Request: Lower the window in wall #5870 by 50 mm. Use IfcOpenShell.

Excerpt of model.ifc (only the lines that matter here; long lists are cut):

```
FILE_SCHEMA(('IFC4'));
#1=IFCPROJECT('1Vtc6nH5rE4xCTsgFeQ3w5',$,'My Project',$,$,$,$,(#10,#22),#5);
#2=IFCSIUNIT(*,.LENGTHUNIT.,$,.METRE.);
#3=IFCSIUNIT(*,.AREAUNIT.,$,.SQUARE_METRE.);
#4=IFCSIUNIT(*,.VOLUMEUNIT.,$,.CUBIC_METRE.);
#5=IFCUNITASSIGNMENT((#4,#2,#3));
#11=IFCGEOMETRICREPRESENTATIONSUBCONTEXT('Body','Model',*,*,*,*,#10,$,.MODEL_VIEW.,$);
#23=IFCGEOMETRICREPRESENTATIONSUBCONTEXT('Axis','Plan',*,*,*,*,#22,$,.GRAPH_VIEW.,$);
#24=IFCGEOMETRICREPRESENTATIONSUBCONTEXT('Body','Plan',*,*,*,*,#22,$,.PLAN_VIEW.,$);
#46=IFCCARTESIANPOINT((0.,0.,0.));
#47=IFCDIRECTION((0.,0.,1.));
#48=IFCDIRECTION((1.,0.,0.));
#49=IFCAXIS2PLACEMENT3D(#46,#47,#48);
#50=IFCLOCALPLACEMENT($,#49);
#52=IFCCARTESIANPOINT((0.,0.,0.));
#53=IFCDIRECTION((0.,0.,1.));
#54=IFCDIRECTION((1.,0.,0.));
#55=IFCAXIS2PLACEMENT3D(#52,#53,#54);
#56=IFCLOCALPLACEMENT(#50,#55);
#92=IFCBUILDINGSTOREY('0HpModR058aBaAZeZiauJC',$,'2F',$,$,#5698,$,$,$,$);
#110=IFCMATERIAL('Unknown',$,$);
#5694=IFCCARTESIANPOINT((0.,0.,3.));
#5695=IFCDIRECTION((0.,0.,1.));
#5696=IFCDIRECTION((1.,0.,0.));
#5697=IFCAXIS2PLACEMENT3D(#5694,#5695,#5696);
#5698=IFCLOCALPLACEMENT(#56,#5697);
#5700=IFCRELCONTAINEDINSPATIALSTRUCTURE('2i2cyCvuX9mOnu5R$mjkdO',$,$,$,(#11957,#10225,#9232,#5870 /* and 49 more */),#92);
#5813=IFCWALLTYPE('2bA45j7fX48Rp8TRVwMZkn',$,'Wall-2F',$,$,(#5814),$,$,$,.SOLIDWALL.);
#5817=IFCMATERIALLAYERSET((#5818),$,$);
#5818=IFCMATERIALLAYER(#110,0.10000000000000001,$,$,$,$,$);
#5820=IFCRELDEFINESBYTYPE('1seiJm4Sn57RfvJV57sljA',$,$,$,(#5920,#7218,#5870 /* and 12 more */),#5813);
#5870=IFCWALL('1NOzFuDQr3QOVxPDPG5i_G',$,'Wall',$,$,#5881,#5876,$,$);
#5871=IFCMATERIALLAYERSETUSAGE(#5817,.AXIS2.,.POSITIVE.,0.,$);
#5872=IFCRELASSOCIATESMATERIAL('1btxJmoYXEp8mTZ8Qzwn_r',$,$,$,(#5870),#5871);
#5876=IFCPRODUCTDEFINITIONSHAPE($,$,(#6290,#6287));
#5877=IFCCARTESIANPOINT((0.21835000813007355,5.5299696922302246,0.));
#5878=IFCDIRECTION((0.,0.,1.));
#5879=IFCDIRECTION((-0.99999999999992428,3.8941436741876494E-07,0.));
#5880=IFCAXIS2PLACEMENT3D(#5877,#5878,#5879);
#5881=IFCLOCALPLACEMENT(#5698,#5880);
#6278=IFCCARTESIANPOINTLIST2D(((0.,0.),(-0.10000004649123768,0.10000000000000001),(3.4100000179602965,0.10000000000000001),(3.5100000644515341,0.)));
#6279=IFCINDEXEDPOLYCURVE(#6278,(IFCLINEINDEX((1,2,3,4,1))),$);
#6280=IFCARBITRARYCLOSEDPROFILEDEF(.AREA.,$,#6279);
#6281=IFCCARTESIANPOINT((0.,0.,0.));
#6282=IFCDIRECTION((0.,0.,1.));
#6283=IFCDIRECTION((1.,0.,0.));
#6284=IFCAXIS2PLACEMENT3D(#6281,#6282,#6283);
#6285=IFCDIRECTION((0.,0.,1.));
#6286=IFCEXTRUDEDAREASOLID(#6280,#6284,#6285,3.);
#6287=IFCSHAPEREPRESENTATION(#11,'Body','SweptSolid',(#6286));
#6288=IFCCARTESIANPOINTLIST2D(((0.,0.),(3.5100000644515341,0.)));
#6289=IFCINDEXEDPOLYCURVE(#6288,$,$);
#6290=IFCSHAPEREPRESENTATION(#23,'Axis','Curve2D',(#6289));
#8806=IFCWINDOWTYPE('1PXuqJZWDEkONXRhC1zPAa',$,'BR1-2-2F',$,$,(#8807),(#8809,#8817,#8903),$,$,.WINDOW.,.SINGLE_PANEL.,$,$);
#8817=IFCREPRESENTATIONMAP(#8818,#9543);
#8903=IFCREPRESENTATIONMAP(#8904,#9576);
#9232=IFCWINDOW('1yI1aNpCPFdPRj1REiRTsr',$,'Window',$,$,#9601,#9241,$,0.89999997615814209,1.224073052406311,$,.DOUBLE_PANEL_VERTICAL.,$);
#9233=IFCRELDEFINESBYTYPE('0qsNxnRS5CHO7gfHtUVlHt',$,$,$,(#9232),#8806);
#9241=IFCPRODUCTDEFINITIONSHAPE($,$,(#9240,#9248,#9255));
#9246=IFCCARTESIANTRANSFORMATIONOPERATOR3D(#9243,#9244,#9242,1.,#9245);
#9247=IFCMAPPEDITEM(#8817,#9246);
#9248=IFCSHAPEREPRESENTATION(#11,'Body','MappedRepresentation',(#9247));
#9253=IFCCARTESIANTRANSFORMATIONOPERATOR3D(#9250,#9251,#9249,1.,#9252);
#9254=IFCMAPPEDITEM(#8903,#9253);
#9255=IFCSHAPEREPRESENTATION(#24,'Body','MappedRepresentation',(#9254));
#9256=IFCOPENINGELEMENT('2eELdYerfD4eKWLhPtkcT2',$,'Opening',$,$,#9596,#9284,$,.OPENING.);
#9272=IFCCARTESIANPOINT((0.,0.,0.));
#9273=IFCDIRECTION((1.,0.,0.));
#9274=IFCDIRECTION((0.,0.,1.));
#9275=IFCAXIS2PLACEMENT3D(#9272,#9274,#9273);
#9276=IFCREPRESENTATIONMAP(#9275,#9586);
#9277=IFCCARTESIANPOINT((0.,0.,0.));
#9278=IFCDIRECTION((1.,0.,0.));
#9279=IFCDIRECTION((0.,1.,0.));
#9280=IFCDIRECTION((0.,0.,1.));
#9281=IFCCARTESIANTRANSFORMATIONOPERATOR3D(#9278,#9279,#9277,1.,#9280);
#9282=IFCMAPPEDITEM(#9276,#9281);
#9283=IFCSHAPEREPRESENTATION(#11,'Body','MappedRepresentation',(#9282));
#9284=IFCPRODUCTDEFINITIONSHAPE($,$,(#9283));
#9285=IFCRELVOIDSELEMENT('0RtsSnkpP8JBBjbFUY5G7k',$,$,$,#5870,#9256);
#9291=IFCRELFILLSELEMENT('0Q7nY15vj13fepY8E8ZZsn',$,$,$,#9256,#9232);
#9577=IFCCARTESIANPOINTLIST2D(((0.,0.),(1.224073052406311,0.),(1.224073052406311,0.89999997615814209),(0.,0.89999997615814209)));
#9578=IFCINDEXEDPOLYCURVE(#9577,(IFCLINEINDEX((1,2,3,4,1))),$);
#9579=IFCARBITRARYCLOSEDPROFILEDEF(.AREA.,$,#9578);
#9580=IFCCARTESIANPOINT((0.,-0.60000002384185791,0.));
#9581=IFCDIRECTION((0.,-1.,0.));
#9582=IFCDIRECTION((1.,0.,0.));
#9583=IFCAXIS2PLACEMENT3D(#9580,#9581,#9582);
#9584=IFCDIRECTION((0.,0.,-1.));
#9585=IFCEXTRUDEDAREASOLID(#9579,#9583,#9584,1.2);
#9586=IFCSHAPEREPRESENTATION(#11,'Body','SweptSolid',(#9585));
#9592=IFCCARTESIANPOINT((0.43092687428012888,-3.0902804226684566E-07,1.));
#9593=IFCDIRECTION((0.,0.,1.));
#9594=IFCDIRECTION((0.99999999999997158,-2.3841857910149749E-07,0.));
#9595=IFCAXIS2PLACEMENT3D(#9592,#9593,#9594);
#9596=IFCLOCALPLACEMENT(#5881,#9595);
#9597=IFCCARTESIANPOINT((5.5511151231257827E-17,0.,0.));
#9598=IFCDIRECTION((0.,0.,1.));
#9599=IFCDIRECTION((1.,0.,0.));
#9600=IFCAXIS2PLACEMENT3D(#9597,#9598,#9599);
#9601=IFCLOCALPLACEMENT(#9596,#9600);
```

```python
import numpy as np
import ifcopenshell
import ifcopenshell.api.geometry
import ifcopenshell.util.placement
import ifcopenshell.util.unit

model = ifcopenshell.open("model.ifc")
unit_scale = ifcopenshell.util.unit.calculate_unit_scale(model)

window = model.by_guid("1yI1aNpCPFdPRj1REiRTsr")
opening = window.FillsVoids[0].RelatingOpeningElement
dz = -0.05

shift = np.array([0.0, 0.0, dz])
# The window is placed relative to its opening, so it follows when the opening moves.
matrix = ifcopenshell.util.placement.get_local_placement(opening.ObjectPlacement)
matrix[:3, 3] += shift
ifcopenshell.api.geometry.edit_object_placement(
    model, product=opening, matrix=matrix, is_si=False, should_transform_children=True
)

print(f"moved by {dz * unit_scale:+.3f} m")

model.write("model-out.ifc")
```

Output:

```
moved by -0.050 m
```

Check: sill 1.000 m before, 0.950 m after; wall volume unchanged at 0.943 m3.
